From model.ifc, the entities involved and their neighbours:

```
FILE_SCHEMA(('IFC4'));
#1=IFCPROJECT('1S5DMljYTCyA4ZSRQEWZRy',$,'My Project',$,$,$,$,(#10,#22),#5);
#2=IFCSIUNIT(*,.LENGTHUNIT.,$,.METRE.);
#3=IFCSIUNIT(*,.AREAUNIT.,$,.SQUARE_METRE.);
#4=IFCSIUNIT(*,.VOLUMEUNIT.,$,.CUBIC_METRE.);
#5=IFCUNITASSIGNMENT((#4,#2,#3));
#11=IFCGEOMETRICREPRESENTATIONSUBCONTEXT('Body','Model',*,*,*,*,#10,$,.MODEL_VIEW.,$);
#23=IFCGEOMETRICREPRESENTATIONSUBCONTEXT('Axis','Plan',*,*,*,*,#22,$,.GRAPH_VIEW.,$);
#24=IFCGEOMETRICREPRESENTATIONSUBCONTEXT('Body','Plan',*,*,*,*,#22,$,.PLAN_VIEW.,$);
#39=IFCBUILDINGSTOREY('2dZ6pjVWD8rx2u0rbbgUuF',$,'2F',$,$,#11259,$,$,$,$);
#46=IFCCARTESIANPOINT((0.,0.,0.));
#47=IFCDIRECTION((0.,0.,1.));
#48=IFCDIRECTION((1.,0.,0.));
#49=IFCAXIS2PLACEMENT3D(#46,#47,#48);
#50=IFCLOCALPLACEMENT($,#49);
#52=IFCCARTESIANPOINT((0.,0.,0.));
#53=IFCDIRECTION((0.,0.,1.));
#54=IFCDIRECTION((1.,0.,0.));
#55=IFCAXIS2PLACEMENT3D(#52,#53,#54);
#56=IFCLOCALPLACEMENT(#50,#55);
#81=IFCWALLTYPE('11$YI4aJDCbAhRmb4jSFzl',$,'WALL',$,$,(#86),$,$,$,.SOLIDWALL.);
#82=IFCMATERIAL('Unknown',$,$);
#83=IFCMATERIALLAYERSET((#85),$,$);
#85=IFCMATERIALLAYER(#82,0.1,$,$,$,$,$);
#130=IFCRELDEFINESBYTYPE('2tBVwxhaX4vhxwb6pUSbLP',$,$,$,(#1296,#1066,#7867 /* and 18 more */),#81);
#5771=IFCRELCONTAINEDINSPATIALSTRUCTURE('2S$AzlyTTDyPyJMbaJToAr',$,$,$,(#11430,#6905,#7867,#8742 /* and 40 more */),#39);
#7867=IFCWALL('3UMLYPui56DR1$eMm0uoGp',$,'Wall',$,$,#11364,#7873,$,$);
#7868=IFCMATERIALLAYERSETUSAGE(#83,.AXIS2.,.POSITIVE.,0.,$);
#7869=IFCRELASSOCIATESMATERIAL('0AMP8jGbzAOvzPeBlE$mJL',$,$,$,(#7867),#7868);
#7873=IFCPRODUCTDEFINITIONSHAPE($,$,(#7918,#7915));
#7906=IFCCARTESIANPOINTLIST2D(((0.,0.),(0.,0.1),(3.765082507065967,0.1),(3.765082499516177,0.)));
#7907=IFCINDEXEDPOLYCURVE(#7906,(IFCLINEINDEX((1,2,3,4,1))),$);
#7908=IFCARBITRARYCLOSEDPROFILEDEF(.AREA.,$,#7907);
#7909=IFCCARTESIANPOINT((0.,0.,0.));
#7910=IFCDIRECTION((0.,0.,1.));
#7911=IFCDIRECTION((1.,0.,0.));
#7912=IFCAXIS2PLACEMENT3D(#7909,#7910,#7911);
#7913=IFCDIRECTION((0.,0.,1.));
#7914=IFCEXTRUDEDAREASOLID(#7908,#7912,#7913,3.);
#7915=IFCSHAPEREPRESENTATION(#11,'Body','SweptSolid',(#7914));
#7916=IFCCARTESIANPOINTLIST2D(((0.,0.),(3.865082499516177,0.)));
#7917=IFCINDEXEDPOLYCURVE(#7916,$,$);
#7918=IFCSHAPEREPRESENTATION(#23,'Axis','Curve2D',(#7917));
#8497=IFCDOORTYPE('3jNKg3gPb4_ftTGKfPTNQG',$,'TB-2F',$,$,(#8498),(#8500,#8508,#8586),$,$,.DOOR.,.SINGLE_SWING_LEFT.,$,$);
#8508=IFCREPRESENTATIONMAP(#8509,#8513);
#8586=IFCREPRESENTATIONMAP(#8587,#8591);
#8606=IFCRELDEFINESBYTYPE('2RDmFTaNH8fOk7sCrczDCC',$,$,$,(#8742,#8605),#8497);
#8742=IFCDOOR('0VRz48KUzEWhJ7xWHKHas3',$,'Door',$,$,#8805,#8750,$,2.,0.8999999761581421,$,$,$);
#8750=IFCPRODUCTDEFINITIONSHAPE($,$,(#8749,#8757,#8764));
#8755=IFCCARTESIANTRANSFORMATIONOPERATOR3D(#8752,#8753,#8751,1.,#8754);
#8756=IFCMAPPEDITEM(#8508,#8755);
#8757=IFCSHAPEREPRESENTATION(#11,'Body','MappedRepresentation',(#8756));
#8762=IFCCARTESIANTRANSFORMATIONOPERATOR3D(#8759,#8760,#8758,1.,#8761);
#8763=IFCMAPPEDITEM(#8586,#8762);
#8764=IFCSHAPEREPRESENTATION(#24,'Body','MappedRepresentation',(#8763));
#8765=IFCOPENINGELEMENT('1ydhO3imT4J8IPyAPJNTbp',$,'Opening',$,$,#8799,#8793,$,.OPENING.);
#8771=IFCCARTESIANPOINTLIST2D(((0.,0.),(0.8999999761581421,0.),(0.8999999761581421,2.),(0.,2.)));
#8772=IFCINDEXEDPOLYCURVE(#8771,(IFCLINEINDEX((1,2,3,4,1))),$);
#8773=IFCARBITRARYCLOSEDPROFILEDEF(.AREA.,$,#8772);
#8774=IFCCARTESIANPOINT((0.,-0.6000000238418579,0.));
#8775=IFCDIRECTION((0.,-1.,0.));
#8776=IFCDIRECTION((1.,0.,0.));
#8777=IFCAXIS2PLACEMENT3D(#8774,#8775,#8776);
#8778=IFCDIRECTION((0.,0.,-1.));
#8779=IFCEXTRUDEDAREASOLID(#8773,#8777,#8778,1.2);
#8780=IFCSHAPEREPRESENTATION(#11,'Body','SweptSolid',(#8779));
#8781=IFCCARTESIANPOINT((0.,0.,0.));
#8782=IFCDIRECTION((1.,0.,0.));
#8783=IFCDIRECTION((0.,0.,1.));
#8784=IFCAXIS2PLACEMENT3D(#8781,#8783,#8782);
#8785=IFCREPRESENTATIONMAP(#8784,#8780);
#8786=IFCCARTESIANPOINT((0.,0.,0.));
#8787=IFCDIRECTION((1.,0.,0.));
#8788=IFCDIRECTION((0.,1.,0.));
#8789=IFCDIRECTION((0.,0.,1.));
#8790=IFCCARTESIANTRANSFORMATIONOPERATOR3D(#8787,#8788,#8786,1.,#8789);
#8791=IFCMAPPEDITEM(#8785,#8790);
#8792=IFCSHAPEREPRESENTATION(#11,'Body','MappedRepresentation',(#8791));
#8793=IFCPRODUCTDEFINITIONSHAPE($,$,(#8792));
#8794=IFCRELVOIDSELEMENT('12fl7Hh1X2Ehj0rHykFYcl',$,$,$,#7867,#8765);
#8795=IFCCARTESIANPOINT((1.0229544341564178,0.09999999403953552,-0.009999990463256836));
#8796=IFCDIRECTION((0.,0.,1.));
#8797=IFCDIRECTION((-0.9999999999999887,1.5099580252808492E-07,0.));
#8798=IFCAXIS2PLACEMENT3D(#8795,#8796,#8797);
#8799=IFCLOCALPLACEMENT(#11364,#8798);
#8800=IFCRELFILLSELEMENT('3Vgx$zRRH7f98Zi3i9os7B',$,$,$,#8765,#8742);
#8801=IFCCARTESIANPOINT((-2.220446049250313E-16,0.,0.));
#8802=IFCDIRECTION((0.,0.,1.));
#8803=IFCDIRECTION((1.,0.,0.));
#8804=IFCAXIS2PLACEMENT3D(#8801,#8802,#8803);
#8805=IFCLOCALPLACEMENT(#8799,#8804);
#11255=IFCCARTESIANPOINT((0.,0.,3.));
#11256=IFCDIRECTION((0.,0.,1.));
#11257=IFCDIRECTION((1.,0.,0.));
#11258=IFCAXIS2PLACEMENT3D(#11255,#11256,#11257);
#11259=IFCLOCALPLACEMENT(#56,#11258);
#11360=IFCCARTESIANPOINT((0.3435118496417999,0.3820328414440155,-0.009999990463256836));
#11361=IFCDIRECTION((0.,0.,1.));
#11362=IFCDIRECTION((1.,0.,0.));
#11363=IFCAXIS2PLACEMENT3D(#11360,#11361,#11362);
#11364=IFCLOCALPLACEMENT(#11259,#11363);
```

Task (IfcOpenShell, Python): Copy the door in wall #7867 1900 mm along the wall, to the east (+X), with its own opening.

```python
import ifcopenshell
import ifcopenshell.api.feature
import ifcopenshell.api.geometry
import ifcopenshell.api.root
import ifcopenshell.geom
import ifcopenshell.util.element
import ifcopenshell.util.placement
import ifcopenshell.util.shape
import ifcopenshell.util.unit

model = ifcopenshell.open("model.ifc")
unit_scale = ifcopenshell.util.unit.calculate_unit_scale(model)
settings = ifcopenshell.geom.settings()


def volume(element):
    """Net volume in cubic metres, openings subtracted."""
    shape = ifcopenshell.geom.create_shape(settings, element)
    return ifcopenshell.util.shape.get_volume(shape.geometry)


door = model.by_guid("0VRz48KUzEWhJ7xWHKHas3")
opening = door.FillsVoids[0].RelatingOpeningElement
wall = opening.VoidsElements[0].RelatingBuildingElement
before = volume(wall)
shift = ifcopenshell.util.placement.get_local_placement(wall.ObjectPlacement)[:3, 0] * 1.9 / unit_scale

# copy_class copies the void relationship, type, container and properties, but no geometry.
new_opening = ifcopenshell.api.root.copy_class(model, product=opening)
new_opening.Representation = ifcopenshell.util.element.copy_deep(
    model, opening.Representation, exclude=["IfcGeometricRepresentationContext", "IfcRepresentationMap"]
)
new_door = ifcopenshell.api.root.copy_class(model, product=door)
new_door.Representation = ifcopenshell.util.element.copy_deep(
    model, door.Representation, exclude=["IfcGeometricRepresentationContext", "IfcRepresentationMap"]
)
ifcopenshell.api.feature.add_filling(model, opening=new_opening, element=new_door)

for old, new in ((opening, new_opening), (door, new_door)):
    matrix = ifcopenshell.util.placement.get_local_placement(old.ObjectPlacement)
    matrix[:3, 3] += shift
    ifcopenshell.api.geometry.edit_object_placement(model, product=new, matrix=matrix, is_si=False)

after = volume(wall)

print(f"wall volume {before:.3f} -> {after:.3f} m3")

model.write("model_rev.ifc")
```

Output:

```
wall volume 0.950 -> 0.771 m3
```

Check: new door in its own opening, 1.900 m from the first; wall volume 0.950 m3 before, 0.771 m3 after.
